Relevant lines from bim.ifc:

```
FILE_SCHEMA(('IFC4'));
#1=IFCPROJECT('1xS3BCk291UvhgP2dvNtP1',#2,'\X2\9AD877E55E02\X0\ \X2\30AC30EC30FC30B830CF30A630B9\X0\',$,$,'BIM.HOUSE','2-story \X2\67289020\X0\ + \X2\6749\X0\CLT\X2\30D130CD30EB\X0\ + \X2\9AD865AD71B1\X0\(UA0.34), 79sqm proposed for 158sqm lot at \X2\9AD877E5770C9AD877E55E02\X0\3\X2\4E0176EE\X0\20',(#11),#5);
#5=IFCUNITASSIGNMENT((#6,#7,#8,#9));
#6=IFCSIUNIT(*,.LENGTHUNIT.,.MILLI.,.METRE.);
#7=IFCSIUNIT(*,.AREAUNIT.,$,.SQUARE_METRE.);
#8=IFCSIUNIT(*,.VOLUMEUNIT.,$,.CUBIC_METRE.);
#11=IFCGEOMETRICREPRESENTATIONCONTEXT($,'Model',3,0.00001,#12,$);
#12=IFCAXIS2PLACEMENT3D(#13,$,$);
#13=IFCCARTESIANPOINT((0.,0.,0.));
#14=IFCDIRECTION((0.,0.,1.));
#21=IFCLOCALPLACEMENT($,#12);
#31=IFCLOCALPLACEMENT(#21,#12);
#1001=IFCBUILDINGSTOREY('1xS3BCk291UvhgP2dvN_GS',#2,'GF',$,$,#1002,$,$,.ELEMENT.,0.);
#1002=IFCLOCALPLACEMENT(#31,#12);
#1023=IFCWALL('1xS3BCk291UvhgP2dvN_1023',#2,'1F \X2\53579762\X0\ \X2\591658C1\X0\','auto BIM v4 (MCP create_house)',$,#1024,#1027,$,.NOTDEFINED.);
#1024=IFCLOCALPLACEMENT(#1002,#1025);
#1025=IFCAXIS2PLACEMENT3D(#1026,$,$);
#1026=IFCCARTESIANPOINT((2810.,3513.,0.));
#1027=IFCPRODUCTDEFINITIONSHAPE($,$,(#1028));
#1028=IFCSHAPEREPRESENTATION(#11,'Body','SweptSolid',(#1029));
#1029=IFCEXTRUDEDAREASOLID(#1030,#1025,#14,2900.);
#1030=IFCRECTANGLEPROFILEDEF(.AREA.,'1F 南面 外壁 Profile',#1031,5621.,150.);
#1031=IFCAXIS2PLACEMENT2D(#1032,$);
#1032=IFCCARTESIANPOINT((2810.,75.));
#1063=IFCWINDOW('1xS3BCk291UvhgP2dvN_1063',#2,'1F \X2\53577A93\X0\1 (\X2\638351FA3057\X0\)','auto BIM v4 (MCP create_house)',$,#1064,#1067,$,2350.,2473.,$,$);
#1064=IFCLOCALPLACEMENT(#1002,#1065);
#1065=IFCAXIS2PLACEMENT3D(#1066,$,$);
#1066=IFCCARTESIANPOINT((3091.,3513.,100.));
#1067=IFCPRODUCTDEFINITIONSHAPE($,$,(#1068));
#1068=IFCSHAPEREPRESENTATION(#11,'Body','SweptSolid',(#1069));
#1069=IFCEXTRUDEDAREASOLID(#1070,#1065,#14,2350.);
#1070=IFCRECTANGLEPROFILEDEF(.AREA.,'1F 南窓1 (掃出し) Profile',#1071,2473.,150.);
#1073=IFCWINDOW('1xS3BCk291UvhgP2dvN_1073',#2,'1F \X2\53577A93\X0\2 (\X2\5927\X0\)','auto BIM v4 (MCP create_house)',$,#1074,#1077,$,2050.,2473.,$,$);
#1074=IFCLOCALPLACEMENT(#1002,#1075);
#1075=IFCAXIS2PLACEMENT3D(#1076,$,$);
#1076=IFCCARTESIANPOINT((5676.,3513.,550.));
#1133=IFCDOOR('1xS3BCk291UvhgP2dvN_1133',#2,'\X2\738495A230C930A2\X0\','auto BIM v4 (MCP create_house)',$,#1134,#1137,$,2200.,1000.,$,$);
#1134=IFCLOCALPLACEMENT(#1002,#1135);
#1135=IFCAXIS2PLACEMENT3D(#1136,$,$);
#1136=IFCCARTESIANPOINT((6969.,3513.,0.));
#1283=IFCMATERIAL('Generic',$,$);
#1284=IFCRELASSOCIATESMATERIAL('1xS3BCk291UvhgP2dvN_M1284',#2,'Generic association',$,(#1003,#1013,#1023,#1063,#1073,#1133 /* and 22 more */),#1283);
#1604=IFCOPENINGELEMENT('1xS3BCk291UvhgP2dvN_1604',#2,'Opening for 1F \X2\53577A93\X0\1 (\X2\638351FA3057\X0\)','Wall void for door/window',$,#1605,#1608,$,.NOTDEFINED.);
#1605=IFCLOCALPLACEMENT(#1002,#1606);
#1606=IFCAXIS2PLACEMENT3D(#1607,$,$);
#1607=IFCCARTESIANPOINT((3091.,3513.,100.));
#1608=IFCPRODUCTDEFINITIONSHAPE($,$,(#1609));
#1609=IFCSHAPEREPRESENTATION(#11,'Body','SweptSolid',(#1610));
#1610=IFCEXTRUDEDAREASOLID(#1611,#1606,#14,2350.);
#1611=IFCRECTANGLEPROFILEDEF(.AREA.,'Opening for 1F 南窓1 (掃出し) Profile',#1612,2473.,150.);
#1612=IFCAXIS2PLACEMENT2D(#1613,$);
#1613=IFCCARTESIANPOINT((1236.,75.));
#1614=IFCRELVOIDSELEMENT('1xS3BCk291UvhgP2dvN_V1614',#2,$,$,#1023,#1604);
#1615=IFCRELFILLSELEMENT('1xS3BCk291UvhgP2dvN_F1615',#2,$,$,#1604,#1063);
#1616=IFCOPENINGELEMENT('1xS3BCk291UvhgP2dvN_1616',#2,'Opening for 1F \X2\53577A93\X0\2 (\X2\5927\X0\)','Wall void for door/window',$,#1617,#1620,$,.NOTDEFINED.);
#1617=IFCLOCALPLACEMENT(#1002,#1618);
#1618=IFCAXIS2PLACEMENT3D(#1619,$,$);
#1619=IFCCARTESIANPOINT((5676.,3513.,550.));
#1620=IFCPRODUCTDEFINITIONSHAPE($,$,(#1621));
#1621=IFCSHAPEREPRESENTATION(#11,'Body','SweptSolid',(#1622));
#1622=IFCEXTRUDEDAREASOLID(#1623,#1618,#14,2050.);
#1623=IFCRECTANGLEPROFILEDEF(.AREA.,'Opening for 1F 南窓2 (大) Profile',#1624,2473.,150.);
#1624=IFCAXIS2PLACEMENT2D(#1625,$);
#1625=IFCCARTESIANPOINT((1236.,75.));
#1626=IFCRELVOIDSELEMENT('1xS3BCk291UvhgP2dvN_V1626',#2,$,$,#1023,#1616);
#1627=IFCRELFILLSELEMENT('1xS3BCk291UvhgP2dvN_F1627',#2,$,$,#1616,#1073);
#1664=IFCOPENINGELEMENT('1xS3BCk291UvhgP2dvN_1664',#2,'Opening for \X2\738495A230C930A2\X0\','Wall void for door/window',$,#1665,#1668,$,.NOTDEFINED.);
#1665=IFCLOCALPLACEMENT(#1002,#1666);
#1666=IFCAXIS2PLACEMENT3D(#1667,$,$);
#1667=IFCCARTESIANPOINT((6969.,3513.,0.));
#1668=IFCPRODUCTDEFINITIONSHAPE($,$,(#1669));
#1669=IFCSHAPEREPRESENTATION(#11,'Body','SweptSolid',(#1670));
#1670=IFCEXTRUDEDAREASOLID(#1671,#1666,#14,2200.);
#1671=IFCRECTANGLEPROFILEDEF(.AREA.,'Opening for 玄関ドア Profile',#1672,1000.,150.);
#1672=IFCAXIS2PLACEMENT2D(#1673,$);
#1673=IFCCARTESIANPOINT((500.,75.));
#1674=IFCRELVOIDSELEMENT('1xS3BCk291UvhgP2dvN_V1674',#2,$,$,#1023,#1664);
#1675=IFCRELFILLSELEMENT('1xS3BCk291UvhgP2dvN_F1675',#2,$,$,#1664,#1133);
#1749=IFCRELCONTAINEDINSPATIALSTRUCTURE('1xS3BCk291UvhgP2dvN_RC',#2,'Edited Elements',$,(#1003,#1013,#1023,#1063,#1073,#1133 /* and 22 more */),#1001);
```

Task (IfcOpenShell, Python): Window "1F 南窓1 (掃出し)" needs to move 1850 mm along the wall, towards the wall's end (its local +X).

```python
import ifcopenshell
import ifcopenshell.api.geometry
import ifcopenshell.util.placement
import ifcopenshell.util.unit

model = ifcopenshell.open("bim.ifc")
unit_scale = ifcopenshell.util.unit.calculate_unit_scale(model)

window = model.by_guid("1xS3BCk291UvhgP2dvN_1063")
opening = window.FillsVoids[0].RelatingOpeningElement
wall = opening.VoidsElements[0].RelatingBuildingElement

wall_matrix = ifcopenshell.util.placement.get_local_placement(wall.ObjectPlacement)
shift = wall_matrix[:3, 0] * 1.85 / unit_scale
before = ifcopenshell.util.placement.get_local_placement(window.ObjectPlacement)[:3, 3].copy()

# The window is not placed relative to its opening, so move both.
for product in (opening, window):
    matrix = ifcopenshell.util.placement.get_local_placement(product.ObjectPlacement)
    matrix[:3, 3] += shift
    ifcopenshell.api.geometry.edit_object_placement(model, product=product, matrix=matrix, is_si=False)

after = ifcopenshell.util.placement.get_local_placement(window.ObjectPlacement)[:3, 3]
print("window moved by", (after - before).round(3) + 0.0)

model.write("bim_edited.ifc")
```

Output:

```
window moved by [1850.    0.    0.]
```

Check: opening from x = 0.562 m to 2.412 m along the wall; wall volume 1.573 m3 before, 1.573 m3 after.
